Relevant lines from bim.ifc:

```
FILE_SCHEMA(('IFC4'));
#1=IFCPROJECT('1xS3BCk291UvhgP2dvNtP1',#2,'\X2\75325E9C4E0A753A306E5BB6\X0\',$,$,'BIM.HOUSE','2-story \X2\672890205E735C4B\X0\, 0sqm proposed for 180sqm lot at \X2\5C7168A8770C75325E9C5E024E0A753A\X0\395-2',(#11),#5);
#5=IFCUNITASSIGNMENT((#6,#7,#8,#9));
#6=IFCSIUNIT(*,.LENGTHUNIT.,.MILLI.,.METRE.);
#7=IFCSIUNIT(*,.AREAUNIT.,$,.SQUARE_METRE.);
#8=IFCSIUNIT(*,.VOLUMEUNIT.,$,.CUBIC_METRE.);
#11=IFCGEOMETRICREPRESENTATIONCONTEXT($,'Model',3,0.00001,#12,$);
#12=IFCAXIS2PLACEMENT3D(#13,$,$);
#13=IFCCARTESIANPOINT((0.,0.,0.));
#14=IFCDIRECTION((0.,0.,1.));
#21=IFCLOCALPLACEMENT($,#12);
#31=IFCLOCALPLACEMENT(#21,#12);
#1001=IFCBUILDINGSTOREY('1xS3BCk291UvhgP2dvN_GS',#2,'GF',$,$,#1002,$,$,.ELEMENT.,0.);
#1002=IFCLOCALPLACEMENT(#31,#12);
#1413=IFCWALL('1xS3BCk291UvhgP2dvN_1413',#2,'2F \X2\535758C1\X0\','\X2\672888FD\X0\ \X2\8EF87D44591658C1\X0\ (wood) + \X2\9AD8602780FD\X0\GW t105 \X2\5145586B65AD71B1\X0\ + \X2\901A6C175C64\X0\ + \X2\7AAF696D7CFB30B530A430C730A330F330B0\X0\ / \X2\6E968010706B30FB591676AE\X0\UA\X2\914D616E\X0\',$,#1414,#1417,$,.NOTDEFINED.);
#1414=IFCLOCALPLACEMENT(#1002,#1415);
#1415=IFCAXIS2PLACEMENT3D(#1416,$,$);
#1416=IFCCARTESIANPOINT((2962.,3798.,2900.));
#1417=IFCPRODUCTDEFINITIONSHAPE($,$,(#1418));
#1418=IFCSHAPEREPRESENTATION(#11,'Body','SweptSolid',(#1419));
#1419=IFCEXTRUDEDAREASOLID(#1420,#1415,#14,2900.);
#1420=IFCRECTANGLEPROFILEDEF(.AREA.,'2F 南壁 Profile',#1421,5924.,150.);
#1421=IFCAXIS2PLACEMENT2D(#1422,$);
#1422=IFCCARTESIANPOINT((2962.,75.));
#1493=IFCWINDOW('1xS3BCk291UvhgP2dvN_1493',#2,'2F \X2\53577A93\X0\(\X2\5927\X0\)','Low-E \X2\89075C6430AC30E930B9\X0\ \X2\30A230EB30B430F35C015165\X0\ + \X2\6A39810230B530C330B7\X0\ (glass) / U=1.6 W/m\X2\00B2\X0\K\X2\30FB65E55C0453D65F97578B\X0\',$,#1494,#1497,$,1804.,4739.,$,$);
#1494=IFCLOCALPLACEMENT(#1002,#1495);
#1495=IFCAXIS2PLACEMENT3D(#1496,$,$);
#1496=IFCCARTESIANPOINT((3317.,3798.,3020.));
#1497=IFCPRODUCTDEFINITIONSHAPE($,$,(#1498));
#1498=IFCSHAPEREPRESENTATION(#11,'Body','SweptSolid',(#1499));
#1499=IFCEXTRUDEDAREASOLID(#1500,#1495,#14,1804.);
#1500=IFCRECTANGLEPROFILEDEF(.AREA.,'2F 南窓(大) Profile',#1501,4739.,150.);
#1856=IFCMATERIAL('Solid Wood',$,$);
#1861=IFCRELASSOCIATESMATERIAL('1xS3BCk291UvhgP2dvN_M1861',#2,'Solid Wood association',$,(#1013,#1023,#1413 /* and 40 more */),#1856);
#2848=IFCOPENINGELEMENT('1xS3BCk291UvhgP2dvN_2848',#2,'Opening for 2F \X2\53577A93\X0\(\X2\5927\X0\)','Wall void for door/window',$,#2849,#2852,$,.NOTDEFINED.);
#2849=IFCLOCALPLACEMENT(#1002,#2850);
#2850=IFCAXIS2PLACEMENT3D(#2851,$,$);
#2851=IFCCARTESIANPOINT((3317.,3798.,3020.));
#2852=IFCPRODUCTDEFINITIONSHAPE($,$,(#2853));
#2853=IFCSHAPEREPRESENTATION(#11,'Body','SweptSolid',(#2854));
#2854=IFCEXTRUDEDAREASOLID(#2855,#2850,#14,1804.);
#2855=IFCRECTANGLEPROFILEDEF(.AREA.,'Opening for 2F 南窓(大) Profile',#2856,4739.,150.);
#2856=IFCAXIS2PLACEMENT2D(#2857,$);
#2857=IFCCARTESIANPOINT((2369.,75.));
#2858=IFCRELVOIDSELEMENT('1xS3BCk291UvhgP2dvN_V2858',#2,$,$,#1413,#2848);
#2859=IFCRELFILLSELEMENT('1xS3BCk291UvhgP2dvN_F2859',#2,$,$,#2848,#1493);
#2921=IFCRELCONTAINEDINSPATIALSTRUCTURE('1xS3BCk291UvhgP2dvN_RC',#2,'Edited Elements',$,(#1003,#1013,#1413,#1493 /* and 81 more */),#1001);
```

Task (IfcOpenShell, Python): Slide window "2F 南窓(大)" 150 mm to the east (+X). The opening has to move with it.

```python
import ifcopenshell
import ifcopenshell.api.geometry
import ifcopenshell.util.placement
import ifcopenshell.util.unit

model = ifcopenshell.open("bim.ifc")
unit_scale = ifcopenshell.util.unit.calculate_unit_scale(model)

window = model.by_guid("1xS3BCk291UvhgP2dvN_1493")
opening = window.FillsVoids[0].RelatingOpeningElement
wall = opening.VoidsElements[0].RelatingBuildingElement

wall_matrix = ifcopenshell.util.placement.get_local_placement(wall.ObjectPlacement)
shift = wall_matrix[:3, 0] * 0.15 / unit_scale
before = ifcopenshell.util.placement.get_local_placement(window.ObjectPlacement)[:3, 3].copy()

# The window is not placed relative to its opening, so move both.
for product in (opening, window):
    matrix = ifcopenshell.util.placement.get_local_placement(product.ObjectPlacement)
    matrix[:3, 3] += shift
    ifcopenshell.api.geometry.edit_object_placement(model, product=product, matrix=matrix, is_si=False)

after = ifcopenshell.util.placement.get_local_placement(window.ObjectPlacement)[:3, 3]
print("window moved by", (after - before).round(3) + 0.0)

model.write("bim_v2.ifc")
```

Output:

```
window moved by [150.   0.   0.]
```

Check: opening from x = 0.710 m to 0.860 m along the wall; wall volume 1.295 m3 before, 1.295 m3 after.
